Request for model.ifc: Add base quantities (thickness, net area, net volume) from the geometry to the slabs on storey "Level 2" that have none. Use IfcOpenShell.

First a look at what the model holds.

```python
import ifcopenshell
import ifcopenshell.util.element
import ifcopenshell.util.unit

model = ifcopenshell.open("model.ifc")
print(model.schema)
for unit_type in ("LENGTHUNIT", "AREAUNIT", "VOLUMEUNIT"):
    print(unit_type, ifcopenshell.util.unit.calculate_unit_scale(model, unit_type))
storey = next(s for s in model.by_type("IfcBuildingStorey") if s.Name == "Level 2")
slabs = [e for e in ifcopenshell.util.element.get_decomposition(storey) if e.is_a("IfcSlab")]
for e in sorted(slabs, key=lambda e: e.id()):
    print(e.id(), e.is_a(), e.Name, list(ifcopenshell.util.element.get_psets(e, qtos_only=True)), sep=" | ")
```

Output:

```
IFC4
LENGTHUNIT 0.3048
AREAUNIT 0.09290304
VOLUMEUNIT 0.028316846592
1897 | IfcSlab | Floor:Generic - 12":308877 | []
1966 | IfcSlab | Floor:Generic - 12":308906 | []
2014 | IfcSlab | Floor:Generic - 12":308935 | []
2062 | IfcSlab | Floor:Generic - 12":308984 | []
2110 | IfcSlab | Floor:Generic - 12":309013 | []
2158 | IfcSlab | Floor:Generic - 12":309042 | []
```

```python
import ifcopenshell
import ifcopenshell.api.pset
import ifcopenshell.geom
import ifcopenshell.util.element
import ifcopenshell.util.shape
import ifcopenshell.util.unit

model = ifcopenshell.open("model.ifc")
unit_scale = ifcopenshell.util.unit.calculate_unit_scale(model)
area_scale = ifcopenshell.util.unit.calculate_unit_scale(model, "AREAUNIT")
volume_scale = ifcopenshell.util.unit.calculate_unit_scale(model, "VOLUMEUNIT")
settings = ifcopenshell.geom.settings()

storey = next(s for s in model.by_type("IfcBuildingStorey") if s.Name == "Level 2")
slabs = [e for e in ifcopenshell.util.element.get_decomposition(storey) if e.is_a("IfcSlab")]

for e in sorted(slabs, key=lambda e: e.id()):
    if ifcopenshell.util.element.get_psets(e, qtos_only=True, should_inherit=False):
        continue
    # Geometry comes back in metres, in the element's own axes.
    shape = ifcopenshell.geom.create_shape(settings, e)
    values = {
        "Width": ifcopenshell.util.shape.get_z(shape.geometry) / unit_scale,
        "NetArea": ifcopenshell.util.shape.get_footprint_area(shape.geometry) / area_scale,
        "NetVolume": ifcopenshell.util.shape.get_volume(shape.geometry) / volume_scale,
    }
    qto = ifcopenshell.api.pset.add_qto(model, product=e, name="Qto_SlabBaseQuantities")
    ifcopenshell.api.pset.edit_qto(model, qto=qto, properties=values)
    print(e.id(), {k: round(v, 3) for k, v in values.items()})

model.write("model_updated.ifc")
```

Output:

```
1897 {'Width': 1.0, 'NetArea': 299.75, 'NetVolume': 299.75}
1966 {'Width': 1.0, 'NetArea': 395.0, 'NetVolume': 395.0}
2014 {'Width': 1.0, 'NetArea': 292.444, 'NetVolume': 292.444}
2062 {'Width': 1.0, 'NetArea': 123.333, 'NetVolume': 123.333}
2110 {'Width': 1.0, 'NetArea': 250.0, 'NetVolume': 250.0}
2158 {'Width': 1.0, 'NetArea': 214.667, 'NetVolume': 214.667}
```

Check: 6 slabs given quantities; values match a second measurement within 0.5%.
